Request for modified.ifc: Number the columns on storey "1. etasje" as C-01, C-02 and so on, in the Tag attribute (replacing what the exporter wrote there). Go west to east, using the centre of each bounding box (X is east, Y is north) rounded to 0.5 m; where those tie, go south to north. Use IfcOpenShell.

First a look at what the model holds.

```python
import ifcopenshell
import ifcopenshell.util.element
import ifcopenshell.util.placement

model = ifcopenshell.open("modified.ifc")
print(model.schema)
storey = next(s for s in model.by_type("IfcBuildingStorey") if s.Name == "1. etasje")
columns = [e for e in ifcopenshell.util.element.get_decomposition(storey) if e.is_a("IfcColumn")]
for e in sorted(columns, key=lambda e: e.id()):
    origin = ifcopenshell.util.placement.get_local_placement(e.ObjectPlacement)[:3, 3]
    print(e.id(), e.Tag, e.Name, origin.round(2) + 0.0, sep=" | ")
```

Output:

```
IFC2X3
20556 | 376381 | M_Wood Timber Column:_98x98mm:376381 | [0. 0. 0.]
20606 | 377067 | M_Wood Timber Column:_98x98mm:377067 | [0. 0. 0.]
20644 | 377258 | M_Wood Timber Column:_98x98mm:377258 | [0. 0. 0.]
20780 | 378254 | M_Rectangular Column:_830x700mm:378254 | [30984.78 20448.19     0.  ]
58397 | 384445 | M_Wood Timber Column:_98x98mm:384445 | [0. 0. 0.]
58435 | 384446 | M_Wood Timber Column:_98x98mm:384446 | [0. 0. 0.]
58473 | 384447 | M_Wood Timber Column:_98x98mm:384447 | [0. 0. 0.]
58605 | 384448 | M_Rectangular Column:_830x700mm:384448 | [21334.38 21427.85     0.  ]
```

```python
import ifcopenshell
import ifcopenshell.geom
import ifcopenshell.util.element
import ifcopenshell.util.shape

model = ifcopenshell.open("modified.ifc")
settings = ifcopenshell.geom.settings()
settings.set("use-world-coords", True)


def centre(element):
    shape = ifcopenshell.geom.create_shape(settings, element)
    return ifcopenshell.util.shape.get_bbox_centroid(shape.geometry)


storey = next(s for s in model.by_type("IfcBuildingStorey") if s.Name == "1. etasje")
columns = [e for e in ifcopenshell.util.element.get_decomposition(storey) if e.is_a("IfcColumn")]

# Insertion points can sit at a corner or the storey origin, so sort by the geometry (in metres).
centres = {e: centre(e) for e in columns}
columns.sort(key=lambda e: (round(centres[e][0] / 0.5), centres[e][1]))

for i, e in enumerate(columns, start=1):
    number = f"C-{i:02d}"
    e.Tag = number
    print(e.id(), number)

model.write("modified_v2.ifc")
```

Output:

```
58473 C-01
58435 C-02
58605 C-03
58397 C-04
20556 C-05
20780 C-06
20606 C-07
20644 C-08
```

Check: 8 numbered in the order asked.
